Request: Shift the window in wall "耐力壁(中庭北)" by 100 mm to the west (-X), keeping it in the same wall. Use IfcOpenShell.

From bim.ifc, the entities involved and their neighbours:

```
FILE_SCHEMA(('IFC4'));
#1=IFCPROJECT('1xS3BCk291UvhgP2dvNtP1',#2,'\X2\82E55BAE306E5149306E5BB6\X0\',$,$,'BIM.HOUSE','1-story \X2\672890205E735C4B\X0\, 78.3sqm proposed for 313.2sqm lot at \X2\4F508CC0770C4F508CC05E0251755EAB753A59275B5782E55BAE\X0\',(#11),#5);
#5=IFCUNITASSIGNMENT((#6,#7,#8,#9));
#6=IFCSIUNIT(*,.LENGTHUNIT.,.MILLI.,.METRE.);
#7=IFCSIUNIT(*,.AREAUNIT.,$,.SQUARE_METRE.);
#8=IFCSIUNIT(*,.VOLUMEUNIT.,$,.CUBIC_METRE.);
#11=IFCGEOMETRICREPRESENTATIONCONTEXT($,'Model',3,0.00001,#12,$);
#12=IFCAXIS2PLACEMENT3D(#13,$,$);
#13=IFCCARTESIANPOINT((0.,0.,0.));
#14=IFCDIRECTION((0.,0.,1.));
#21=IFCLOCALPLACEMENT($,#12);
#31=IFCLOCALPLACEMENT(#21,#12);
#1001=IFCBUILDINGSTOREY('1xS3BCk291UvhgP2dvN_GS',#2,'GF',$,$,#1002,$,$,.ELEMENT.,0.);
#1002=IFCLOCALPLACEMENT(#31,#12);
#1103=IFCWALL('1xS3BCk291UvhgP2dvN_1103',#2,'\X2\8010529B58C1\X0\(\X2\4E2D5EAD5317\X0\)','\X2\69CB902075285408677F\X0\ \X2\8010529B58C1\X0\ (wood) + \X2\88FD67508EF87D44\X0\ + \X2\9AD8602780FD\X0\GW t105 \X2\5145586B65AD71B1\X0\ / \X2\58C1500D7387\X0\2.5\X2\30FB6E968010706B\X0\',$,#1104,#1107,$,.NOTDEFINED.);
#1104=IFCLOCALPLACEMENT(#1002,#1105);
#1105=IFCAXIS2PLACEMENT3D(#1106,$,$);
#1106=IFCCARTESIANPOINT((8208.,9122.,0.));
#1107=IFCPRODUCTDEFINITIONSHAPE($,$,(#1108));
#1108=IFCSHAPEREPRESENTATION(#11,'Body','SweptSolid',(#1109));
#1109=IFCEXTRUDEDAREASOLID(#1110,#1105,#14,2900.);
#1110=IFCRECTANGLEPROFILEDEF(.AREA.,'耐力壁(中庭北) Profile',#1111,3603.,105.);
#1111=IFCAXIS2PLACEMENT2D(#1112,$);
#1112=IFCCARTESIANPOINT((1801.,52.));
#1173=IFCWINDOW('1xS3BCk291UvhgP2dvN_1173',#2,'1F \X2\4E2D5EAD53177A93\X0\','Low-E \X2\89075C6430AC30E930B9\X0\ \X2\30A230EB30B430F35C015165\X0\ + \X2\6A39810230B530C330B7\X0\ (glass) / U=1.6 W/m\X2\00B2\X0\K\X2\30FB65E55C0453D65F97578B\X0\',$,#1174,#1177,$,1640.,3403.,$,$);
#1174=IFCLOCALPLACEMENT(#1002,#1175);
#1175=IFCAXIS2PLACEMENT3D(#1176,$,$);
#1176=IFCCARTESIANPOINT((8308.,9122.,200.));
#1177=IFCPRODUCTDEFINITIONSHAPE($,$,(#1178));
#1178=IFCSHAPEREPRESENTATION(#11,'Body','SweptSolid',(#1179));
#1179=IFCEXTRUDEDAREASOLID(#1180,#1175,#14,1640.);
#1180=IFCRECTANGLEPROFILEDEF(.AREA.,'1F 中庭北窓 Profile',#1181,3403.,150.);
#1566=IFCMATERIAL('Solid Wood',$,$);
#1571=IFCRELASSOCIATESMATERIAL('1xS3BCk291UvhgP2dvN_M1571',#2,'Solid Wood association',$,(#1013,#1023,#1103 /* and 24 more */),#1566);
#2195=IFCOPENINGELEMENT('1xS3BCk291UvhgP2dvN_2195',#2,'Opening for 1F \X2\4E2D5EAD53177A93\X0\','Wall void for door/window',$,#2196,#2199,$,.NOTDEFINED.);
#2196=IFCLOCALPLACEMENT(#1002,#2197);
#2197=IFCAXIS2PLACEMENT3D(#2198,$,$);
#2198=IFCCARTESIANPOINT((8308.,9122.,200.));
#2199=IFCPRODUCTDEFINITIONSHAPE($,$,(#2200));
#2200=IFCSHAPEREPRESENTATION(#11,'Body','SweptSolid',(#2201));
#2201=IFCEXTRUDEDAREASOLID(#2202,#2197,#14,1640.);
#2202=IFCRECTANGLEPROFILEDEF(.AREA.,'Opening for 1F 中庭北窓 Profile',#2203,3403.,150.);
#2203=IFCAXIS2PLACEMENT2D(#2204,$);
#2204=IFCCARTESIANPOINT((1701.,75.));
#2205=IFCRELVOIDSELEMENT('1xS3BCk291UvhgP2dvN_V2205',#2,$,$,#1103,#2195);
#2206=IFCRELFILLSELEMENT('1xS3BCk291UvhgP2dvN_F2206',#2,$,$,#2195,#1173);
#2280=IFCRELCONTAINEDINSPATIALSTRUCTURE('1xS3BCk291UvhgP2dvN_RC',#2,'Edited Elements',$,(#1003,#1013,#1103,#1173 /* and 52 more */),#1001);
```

```python
import ifcopenshell
import ifcopenshell.api.geometry
import ifcopenshell.util.placement

model = ifcopenshell.open("bim.ifc")

window = model.by_guid("1xS3BCk291UvhgP2dvN_1173")
opening = window.FillsVoids[0].RelatingOpeningElement
wall = opening.VoidsElements[0].RelatingBuildingElement

wall_matrix = ifcopenshell.util.placement.get_local_placement(wall.ObjectPlacement)
shift = wall_matrix[:3, 0] * -100.0
before = ifcopenshell.util.placement.get_local_placement(window.ObjectPlacement)[:3, 3].copy()

# The window is not placed relative to its opening, so move both.
for product in (opening, window):
    matrix = ifcopenshell.util.placement.get_local_placement(product.ObjectPlacement)
    matrix[:3, 3] += shift
    ifcopenshell.api.geometry.edit_object_placement(model, product=product, matrix=matrix, is_si=False)

after = ifcopenshell.util.placement.get_local_placement(window.ObjectPlacement)[:3, 3]
print("window moved by", (after - before).round(3) + 0.0)

model.write("bim-out.ifc")
```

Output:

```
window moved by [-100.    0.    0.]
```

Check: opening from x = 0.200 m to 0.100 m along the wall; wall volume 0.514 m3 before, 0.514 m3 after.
